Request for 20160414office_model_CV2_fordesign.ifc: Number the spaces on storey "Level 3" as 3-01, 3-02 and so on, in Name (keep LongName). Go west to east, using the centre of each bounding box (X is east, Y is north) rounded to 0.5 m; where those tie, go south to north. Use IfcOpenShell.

First a look at what the model holds.

```python
import ifcopenshell
import ifcopenshell.util.element
import ifcopenshell.util.placement

model = ifcopenshell.open("20160414office_model_CV2_fordesign.ifc")
print(model.schema)
storey = next(s for s in model.by_type("IfcBuildingStorey") if s.Name == "Level 3")
spaces = [e for e in ifcopenshell.util.element.get_decomposition(storey) if e.is_a("IfcSpace")]
for e in sorted(spaces, key=lambda e: e.id()):
    origin = ifcopenshell.util.placement.get_local_placement(e.ObjectPlacement)[:3, 3]
    print(e.id(), e.Name, e.LongName, origin.round(2) + 0.0, sep=" | ")
```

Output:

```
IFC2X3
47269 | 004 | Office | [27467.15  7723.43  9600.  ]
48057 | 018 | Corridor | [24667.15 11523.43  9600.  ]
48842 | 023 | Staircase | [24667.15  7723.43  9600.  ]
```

```python
import ifcopenshell
import ifcopenshell.geom
import ifcopenshell.util.element
import ifcopenshell.util.shape

model = ifcopenshell.open("20160414office_model_CV2_fordesign.ifc")
settings = ifcopenshell.geom.settings()
settings.set("use-world-coords", True)


def centre(element):
    shape = ifcopenshell.geom.create_shape(settings, element)
    return ifcopenshell.util.shape.get_bbox_centroid(shape.geometry)


storey = next(s for s in model.by_type("IfcBuildingStorey") if s.Name == "Level 3")
spaces = [e for e in ifcopenshell.util.element.get_decomposition(storey) if e.is_a("IfcSpace")]

# Insertion points can sit at a corner or the storey origin, so sort by the geometry (in metres).
centres = {e: centre(e) for e in spaces}
spaces.sort(key=lambda e: (round(centres[e][0] / 0.5), centres[e][1]))

for i, e in enumerate(spaces, start=1):
    number = f"3-{i:02d}"
    e.Name = number
    print(e.id(), number)

model.write("20160414office_model_CV2_fordesign_v2.ifc")
```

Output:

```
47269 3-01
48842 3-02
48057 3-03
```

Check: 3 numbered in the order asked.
